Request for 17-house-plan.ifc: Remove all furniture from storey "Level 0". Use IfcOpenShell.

First a look at what the model holds.

```python
import ifcopenshell
import ifcopenshell.util.element

model = ifcopenshell.open("17-house-plan.ifc")
print(model.schema)
storey = next(s for s in model.by_type("IfcBuildingStorey") if s.Name == "Level 0")
furniture = [e for e in ifcopenshell.util.element.get_decomposition(storey) if e.is_a("IfcFurnishingElement")]
seen = {}
for e in furniture:
    element_type = ifcopenshell.util.element.get_type(e)
    name = element_type.Name if element_type not in (None, e) else None
    seen[name] = seen.get(name, 0) + 1
for name, count in sorted(seen.items(), key=str):
    print(count, "x", name)
```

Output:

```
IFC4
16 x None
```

```python
import ifcopenshell
import ifcopenshell.api.root
import ifcopenshell.util.element

model = ifcopenshell.open("17-house-plan.ifc")

storey = next(s for s in model.by_type("IfcBuildingStorey") if s.Name == "Level 0")
furniture = [e for e in ifcopenshell.util.element.get_decomposition(storey) if e.is_a("IfcFurnishingElement")]

for e in furniture:
    ifcopenshell.api.root.remove_product(model, product=e)
print(len(furniture), "removed")

model.write("17-house-plan-out.ifc")
```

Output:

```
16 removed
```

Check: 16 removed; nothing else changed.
